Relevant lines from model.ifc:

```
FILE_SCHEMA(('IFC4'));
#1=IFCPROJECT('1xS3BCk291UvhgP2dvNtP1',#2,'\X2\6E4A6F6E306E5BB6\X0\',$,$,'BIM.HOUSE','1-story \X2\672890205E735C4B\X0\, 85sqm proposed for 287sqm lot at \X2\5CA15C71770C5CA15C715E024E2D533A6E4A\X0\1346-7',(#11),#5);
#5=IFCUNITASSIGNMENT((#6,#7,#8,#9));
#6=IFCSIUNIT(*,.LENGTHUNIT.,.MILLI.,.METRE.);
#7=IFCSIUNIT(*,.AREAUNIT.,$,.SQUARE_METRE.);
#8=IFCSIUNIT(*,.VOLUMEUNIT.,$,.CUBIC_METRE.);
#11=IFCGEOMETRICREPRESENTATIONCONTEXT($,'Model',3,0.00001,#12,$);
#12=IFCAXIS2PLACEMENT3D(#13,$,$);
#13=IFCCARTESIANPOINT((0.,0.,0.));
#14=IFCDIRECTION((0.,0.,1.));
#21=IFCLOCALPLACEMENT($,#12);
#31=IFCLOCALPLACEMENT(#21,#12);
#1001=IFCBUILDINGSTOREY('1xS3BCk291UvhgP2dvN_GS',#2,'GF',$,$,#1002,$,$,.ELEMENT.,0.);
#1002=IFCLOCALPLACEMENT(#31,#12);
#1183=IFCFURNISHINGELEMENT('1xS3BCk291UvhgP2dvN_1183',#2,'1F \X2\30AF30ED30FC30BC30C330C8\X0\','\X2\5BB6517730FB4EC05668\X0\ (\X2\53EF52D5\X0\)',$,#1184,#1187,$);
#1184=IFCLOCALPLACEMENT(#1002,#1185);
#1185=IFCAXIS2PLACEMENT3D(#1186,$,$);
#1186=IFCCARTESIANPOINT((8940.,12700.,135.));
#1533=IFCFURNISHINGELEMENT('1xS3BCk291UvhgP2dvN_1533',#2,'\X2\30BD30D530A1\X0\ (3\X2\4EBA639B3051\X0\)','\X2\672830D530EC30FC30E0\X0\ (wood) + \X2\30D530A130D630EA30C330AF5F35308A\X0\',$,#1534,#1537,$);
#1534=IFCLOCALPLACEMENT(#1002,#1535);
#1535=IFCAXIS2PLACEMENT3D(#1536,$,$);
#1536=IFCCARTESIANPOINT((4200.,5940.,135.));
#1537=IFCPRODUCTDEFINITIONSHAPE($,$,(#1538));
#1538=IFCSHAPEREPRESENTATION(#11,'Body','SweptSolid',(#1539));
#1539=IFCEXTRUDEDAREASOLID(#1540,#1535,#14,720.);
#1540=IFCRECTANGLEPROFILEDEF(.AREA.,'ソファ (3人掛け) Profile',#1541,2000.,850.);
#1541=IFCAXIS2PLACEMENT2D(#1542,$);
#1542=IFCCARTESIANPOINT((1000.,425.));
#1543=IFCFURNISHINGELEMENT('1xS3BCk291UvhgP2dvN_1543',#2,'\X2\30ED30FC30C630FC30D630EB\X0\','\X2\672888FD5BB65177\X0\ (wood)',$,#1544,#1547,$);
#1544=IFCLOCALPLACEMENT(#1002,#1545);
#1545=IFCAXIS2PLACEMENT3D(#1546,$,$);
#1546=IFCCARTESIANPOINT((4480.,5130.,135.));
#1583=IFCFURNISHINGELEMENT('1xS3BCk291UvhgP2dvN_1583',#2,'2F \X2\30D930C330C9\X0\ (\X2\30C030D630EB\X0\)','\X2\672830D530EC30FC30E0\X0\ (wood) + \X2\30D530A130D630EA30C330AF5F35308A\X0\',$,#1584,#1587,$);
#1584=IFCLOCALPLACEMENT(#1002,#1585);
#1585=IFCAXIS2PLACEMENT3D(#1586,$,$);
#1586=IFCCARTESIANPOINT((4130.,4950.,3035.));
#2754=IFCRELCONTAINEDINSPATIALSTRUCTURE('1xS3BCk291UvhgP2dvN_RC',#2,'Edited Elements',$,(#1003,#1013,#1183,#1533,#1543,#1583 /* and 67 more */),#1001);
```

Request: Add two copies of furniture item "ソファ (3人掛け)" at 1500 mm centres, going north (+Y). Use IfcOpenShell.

```python
import numpy as np
import ifcopenshell
import ifcopenshell.api.geometry
import ifcopenshell.api.root
import ifcopenshell.util.element
import ifcopenshell.util.placement
import ifcopenshell.util.unit

model = ifcopenshell.open("model.ifc")
unit_scale = ifcopenshell.util.unit.calculate_unit_scale(model)


def reuse_history(source, copy):
    """copy_class also copies each property set's owner history, people and application; keep the originals."""
    for rel in copy.IsDefinedBy:
        if rel.is_a("IfcRelDefinesByProperties") and (history := rel.RelatingPropertyDefinition.OwnerHistory):
            rel.RelatingPropertyDefinition.OwnerHistory = source.OwnerHistory
            ifcopenshell.util.element.remove_deep2(model, history)


source = model.by_id(1533)
base = ifcopenshell.util.placement.get_local_placement(source.ObjectPlacement)
step = np.array([0.0, 1.0, 0.0]) * 1.5 / unit_scale

for i in range(1, 3):
    copy = ifcopenshell.api.root.copy_class(model, product=source)
    copy.Representation = ifcopenshell.util.element.copy_deep(
        model, source.Representation, exclude=["IfcGeometricRepresentationContext", "IfcRepresentationMap"]
    )
    reuse_history(source, copy)
    matrix = base.copy()
    matrix[:3, 3] += i * step
    print("added at", matrix[:3, 3].round(3) + 0.0)
    ifcopenshell.api.geometry.edit_object_placement(model, product=copy, matrix=matrix, is_si=False)

model.write("model_updated.ifc")
```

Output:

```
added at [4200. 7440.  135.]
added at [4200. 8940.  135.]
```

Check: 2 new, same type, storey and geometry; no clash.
